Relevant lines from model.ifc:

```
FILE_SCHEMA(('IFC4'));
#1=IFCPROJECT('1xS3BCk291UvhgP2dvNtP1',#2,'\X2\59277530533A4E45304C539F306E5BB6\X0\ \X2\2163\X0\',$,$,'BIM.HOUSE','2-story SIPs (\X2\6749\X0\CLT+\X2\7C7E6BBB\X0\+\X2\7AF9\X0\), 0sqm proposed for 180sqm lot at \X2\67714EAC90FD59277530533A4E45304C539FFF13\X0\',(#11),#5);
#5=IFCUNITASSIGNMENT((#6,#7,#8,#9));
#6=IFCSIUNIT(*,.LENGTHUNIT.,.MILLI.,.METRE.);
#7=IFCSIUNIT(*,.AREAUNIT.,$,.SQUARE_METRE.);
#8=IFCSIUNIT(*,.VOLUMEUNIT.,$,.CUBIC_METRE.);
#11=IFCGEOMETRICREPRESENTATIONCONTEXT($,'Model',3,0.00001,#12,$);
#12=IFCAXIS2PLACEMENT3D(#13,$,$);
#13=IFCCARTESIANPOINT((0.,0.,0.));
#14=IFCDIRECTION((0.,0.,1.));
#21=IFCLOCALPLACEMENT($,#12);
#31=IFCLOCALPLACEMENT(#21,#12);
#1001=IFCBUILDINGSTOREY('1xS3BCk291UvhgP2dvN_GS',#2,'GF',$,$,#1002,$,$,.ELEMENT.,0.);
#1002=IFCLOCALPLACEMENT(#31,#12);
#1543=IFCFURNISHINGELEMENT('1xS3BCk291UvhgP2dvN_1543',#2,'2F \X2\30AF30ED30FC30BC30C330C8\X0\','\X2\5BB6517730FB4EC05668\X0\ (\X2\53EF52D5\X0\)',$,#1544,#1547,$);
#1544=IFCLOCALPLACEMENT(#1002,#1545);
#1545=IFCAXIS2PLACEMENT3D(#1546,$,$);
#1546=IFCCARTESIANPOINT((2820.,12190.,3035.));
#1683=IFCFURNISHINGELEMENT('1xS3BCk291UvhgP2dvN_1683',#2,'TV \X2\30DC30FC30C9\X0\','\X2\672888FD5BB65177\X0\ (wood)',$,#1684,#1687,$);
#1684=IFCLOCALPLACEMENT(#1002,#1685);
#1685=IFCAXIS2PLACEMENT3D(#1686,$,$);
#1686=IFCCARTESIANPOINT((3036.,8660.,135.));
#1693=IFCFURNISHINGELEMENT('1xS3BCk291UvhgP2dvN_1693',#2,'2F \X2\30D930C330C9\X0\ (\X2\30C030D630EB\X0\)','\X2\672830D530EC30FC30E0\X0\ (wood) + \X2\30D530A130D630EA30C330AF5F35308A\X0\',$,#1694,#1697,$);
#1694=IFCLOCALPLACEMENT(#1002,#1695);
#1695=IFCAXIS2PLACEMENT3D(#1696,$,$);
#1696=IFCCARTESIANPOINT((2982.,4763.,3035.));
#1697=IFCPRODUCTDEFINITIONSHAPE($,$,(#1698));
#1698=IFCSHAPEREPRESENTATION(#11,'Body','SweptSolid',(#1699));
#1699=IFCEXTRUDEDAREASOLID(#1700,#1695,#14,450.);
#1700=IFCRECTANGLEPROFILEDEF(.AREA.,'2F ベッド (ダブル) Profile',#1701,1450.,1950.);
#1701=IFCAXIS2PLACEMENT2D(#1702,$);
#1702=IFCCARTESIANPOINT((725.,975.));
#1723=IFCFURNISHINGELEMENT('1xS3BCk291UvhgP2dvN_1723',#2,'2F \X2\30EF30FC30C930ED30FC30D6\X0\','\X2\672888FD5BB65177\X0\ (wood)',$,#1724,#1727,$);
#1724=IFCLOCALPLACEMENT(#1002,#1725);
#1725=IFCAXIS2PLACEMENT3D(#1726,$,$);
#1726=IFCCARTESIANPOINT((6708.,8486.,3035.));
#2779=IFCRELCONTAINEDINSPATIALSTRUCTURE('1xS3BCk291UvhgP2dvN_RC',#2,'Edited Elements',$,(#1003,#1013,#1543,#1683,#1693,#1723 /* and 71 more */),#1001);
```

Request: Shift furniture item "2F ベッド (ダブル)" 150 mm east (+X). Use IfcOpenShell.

```python
import ifcopenshell
import ifcopenshell.api.geometry
import ifcopenshell.util.placement
import ifcopenshell.util.unit

model = ifcopenshell.open("model.ifc")
unit_scale = ifcopenshell.util.unit.calculate_unit_scale(model)

item = model.by_guid("1xS3BCk291UvhgP2dvN_1693")
matrix = ifcopenshell.util.placement.get_local_placement(item.ObjectPlacement)
matrix[0, 3] += 0.15 / unit_scale
ifcopenshell.api.geometry.edit_object_placement(model, product=item, matrix=matrix, is_si=False)

print(ifcopenshell.util.placement.get_local_placement(item.ObjectPlacement).round(3) + 0.0)

model.write("model_edited.ifc")
```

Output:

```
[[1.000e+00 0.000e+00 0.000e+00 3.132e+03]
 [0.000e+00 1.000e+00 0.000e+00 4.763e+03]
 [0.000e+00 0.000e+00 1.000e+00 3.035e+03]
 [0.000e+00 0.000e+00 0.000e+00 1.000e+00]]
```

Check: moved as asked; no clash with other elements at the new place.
